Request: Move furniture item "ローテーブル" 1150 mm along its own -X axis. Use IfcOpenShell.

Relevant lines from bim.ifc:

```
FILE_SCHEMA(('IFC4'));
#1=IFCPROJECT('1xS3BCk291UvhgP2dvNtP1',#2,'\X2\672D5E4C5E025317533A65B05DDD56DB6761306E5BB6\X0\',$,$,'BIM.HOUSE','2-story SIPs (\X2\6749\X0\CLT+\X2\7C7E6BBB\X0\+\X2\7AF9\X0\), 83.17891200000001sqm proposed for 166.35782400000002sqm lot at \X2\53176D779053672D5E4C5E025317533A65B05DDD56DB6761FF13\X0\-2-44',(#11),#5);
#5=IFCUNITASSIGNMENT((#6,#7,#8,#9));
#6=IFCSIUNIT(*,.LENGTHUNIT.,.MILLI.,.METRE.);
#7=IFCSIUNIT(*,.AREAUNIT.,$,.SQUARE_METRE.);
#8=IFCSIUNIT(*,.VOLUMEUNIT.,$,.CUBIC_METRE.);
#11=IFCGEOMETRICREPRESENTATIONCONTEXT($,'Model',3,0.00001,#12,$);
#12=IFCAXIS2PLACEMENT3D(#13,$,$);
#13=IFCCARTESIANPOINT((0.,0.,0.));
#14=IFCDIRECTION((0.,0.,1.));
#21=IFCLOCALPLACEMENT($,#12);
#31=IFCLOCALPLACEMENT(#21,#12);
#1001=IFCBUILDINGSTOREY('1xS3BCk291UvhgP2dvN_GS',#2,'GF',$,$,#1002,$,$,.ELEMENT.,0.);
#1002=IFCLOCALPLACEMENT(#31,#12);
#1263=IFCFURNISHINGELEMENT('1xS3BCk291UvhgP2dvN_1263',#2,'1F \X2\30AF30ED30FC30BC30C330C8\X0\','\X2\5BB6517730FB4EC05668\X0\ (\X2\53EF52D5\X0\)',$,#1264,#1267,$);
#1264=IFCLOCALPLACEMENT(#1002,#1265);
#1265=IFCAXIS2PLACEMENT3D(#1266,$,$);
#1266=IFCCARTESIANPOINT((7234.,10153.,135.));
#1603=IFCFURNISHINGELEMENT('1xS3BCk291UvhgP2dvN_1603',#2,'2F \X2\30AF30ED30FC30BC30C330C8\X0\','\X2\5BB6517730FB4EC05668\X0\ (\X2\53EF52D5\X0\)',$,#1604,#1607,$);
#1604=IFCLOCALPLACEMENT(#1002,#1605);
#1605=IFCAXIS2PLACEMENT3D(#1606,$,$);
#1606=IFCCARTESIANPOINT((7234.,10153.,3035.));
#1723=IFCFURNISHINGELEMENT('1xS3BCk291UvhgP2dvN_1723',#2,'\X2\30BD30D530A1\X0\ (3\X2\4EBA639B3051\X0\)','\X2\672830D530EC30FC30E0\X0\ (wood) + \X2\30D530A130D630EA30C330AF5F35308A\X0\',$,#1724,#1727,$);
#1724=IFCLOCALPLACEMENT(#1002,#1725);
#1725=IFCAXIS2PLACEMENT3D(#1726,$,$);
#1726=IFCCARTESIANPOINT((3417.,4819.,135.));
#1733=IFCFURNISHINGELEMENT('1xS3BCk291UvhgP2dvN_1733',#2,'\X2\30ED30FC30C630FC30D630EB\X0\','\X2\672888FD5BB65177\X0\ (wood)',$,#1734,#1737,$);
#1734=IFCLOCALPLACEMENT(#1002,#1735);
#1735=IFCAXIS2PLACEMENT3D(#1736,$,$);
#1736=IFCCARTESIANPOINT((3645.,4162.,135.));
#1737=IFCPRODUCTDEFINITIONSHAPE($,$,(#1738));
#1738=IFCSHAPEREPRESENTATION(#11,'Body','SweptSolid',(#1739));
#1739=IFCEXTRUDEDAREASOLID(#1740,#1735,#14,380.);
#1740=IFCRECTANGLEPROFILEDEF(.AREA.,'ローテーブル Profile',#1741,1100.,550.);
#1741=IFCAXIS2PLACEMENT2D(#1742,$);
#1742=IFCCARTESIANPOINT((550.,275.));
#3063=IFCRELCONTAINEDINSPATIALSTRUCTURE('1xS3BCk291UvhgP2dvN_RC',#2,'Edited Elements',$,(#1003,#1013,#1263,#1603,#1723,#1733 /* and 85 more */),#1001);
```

```python
import ifcopenshell
import ifcopenshell.api.geometry
import ifcopenshell.util.placement

model = ifcopenshell.open("bim.ifc")

item = model.by_guid("1xS3BCk291UvhgP2dvN_1733")
matrix = ifcopenshell.util.placement.get_local_placement(item.ObjectPlacement)
matrix[:3, 3] -= matrix[:3, 0] * 1150.0
ifcopenshell.api.geometry.edit_object_placement(model, product=item, matrix=matrix, is_si=False)

print(ifcopenshell.util.placement.get_local_placement(item.ObjectPlacement).round(3) + 0.0)

model.write("bim-out.ifc")
```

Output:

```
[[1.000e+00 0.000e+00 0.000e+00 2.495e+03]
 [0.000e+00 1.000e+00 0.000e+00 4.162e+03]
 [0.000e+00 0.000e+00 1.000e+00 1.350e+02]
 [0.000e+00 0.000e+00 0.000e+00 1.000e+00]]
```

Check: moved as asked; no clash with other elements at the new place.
